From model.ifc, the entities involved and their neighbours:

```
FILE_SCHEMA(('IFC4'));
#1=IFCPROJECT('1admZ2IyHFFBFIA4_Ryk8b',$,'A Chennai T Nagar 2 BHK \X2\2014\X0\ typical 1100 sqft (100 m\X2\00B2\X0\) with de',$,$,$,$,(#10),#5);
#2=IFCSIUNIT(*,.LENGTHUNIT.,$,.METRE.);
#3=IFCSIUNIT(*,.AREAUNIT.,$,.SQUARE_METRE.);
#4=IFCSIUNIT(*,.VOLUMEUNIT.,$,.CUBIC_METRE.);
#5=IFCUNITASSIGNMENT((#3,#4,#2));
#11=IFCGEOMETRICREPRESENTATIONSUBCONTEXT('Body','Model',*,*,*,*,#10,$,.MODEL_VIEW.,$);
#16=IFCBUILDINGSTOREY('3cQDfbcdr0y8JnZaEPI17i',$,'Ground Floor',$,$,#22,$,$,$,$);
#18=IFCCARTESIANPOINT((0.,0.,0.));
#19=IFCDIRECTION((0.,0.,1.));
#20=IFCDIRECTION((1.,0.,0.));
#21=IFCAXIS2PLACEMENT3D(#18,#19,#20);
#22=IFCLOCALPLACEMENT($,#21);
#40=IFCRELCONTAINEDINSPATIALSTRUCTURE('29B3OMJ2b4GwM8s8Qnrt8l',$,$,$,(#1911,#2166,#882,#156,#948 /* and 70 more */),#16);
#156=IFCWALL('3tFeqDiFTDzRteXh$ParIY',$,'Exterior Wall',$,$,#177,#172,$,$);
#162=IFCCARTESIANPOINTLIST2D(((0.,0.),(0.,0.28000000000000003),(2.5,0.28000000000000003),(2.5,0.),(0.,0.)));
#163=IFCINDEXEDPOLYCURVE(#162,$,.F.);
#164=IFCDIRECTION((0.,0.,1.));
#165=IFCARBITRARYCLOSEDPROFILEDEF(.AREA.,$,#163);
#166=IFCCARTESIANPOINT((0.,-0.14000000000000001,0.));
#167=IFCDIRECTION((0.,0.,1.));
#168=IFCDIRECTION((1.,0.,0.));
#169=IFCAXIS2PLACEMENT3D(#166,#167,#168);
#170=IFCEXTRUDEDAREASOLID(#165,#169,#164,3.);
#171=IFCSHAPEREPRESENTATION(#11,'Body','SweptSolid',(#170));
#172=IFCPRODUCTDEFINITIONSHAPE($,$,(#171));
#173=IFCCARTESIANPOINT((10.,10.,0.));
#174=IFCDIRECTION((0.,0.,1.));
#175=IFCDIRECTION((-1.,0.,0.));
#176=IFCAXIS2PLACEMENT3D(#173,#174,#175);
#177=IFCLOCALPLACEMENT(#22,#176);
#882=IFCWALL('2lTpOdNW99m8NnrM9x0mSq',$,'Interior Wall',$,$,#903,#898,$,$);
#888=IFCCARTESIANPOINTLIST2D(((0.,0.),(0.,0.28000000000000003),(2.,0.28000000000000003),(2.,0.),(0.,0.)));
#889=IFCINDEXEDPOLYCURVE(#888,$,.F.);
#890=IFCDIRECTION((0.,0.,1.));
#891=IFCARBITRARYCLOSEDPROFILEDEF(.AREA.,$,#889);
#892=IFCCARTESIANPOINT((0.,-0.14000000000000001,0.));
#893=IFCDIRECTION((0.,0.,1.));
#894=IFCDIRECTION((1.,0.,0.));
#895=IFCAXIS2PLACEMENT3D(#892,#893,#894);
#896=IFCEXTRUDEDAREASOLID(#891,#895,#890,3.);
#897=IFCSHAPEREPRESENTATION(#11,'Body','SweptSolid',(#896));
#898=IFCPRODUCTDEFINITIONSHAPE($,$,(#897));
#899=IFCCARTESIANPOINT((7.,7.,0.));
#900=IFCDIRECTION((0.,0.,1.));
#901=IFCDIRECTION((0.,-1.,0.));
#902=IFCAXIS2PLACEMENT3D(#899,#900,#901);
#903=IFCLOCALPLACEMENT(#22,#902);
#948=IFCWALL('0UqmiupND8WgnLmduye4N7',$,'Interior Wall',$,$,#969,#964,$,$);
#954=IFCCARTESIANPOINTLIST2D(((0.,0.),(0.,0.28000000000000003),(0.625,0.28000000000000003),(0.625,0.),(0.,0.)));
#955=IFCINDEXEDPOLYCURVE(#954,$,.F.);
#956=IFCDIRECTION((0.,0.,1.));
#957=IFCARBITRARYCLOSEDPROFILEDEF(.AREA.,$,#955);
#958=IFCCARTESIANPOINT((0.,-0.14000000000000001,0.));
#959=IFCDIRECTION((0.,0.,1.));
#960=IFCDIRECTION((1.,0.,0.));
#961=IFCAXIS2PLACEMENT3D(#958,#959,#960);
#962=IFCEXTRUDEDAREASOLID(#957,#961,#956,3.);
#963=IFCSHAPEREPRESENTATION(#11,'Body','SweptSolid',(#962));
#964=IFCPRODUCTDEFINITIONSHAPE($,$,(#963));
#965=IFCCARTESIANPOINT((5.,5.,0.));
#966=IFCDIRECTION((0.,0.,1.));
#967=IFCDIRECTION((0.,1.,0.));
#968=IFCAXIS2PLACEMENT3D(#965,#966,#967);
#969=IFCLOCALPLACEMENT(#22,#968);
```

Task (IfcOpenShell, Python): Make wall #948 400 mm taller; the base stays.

```python
import ifcopenshell
import ifcopenshell.geom
import ifcopenshell.util.representation
import ifcopenshell.util.shape

model = ifcopenshell.open("model.ifc")
settings = ifcopenshell.geom.settings()


def volume(element):
    """Net volume in cubic metres, openings subtracted."""
    shape = ifcopenshell.geom.create_shape(settings, element)
    return ifcopenshell.util.shape.get_volume(shape.geometry)


wall = model.by_id(948)
before = volume(wall)

body = ifcopenshell.util.representation.get_representation(wall, "Model", "Body")
solid = body.Items[0]
old_height = solid.Depth
solid.Depth += 0.4
after = volume(wall)

print(f"height {old_height:g} -> {solid.Depth:g}, volume {before:.3f} -> {after:.3f} m3")

model.write("model-out.ifc")
```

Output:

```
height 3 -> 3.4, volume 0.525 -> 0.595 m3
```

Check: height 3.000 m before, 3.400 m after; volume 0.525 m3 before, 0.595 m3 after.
